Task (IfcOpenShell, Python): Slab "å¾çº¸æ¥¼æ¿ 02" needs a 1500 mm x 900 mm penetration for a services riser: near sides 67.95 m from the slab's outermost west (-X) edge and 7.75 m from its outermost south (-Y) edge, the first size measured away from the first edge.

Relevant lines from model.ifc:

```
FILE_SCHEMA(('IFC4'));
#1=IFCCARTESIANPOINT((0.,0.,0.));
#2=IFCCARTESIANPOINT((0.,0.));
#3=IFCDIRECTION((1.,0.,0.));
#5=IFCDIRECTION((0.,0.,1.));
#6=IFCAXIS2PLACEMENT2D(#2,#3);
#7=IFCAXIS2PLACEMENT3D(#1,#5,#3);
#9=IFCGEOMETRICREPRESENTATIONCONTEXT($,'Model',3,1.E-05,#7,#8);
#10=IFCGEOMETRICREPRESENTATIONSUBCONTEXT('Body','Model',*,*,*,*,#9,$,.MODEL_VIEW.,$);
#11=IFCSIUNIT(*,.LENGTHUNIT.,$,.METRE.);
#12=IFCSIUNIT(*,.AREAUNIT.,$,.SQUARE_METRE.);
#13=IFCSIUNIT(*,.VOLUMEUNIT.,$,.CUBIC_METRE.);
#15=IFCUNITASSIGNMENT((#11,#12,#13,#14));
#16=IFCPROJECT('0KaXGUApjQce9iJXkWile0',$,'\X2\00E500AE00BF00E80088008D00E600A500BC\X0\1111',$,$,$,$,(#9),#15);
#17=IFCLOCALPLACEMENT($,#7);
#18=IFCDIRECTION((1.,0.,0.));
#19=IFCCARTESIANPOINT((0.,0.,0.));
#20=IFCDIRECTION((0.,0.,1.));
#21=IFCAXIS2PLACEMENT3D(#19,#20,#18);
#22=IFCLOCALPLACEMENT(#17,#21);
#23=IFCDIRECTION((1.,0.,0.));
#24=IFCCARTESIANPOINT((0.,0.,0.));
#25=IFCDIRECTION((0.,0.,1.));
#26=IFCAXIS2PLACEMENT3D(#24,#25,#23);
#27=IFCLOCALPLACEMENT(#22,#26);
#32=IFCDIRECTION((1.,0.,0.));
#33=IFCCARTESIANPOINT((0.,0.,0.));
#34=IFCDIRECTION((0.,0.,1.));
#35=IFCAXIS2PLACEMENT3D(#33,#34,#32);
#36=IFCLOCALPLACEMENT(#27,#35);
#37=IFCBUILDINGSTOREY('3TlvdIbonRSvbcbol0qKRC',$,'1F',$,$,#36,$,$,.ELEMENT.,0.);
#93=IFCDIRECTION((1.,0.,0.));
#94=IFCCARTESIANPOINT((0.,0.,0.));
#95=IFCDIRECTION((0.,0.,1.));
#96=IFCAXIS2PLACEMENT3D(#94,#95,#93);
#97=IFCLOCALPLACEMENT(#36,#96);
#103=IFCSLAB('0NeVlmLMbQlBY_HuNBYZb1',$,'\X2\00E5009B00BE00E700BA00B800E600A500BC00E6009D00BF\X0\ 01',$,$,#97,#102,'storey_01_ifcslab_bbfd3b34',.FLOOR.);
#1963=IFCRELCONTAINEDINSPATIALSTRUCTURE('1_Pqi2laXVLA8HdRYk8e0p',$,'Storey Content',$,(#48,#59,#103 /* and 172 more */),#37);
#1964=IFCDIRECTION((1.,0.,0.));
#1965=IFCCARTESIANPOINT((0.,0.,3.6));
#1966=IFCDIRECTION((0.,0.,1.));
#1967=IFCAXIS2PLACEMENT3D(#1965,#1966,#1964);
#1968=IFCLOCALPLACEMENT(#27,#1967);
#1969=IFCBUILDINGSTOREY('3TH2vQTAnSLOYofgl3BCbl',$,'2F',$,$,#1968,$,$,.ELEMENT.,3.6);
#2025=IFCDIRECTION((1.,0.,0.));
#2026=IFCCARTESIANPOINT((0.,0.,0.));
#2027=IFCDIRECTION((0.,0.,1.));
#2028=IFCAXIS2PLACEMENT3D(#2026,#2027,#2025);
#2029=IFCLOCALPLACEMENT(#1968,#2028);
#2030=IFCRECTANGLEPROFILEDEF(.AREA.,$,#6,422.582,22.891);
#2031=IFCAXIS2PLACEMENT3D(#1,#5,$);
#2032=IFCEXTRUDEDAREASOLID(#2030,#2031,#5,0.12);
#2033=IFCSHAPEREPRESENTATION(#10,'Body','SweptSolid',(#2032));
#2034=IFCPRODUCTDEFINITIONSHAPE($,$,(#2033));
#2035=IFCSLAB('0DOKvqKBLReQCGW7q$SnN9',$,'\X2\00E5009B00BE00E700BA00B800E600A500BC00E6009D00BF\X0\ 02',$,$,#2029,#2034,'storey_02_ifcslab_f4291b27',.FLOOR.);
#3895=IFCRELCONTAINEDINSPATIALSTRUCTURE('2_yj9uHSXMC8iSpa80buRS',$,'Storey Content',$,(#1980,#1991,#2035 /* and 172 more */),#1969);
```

```python
import numpy as np
import ifcopenshell
import ifcopenshell.api.feature
import ifcopenshell.api.geometry
import ifcopenshell.api.root
import ifcopenshell.geom
import ifcopenshell.util.placement
import ifcopenshell.util.representation
import ifcopenshell.util.shape
import ifcopenshell.util.unit

model = ifcopenshell.open("model.ifc")
unit_scale = ifcopenshell.util.unit.calculate_unit_scale(model)
settings = ifcopenshell.geom.settings()


def volume(element):
    """Net volume in cubic metres, openings subtracted."""
    shape = ifcopenshell.geom.create_shape(settings, element)
    return ifcopenshell.util.shape.get_volume(shape.geometry)


slab = model.by_id(2035)
before = volume(slab)

# Extent in the slab's own axes, in metres. The edges named are its -X and -Y sides.
slab_shape = ifcopenshell.geom.create_shape(settings, slab)
vertices = ifcopenshell.util.shape.get_vertices(slab_shape.geometry)
x_min, y_min, bottom = vertices.min(axis=0)
top = vertices[:, 2].max()

opening = ifcopenshell.api.root.create_entity(model, ifc_class="IfcOpeningElement", name="Services riser opening", predefined_type="OPENING")
context = ifcopenshell.util.representation.get_context(model, "Model", "Body", "MODEL_VIEW")
width, depth = 1.5, 0.9
outline = [(0.0, 0.0), (width, 0.0), (width, depth), (0.0, depth), (0.0, 0.0)]
# Overshoot both faces by 50 mm so the cut is clean.
shape = ifcopenshell.api.geometry.add_slab_representation(
    model, context=context, depth=top - bottom + 0.1, polyline=outline
)
ifcopenshell.api.geometry.assign_representation(model, product=opening, representation=shape)

matrix = ifcopenshell.util.placement.get_local_placement(slab.ObjectPlacement)
matrix[:, 3] = matrix @ np.append(np.array([x_min + 67.95, y_min + 7.75, bottom - 0.05]) / unit_scale, 1.0)
ifcopenshell.api.geometry.edit_object_placement(model, product=opening, matrix=matrix, is_si=False)
ifcopenshell.api.feature.add_feature(model, feature=opening, element=slab)

after = volume(slab)

print(f"slab volume {before:.3f} -> {after:.3f} m3")

model.write("model_updated.ifc")
```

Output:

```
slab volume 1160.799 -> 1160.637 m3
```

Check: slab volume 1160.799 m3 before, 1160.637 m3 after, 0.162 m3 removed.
